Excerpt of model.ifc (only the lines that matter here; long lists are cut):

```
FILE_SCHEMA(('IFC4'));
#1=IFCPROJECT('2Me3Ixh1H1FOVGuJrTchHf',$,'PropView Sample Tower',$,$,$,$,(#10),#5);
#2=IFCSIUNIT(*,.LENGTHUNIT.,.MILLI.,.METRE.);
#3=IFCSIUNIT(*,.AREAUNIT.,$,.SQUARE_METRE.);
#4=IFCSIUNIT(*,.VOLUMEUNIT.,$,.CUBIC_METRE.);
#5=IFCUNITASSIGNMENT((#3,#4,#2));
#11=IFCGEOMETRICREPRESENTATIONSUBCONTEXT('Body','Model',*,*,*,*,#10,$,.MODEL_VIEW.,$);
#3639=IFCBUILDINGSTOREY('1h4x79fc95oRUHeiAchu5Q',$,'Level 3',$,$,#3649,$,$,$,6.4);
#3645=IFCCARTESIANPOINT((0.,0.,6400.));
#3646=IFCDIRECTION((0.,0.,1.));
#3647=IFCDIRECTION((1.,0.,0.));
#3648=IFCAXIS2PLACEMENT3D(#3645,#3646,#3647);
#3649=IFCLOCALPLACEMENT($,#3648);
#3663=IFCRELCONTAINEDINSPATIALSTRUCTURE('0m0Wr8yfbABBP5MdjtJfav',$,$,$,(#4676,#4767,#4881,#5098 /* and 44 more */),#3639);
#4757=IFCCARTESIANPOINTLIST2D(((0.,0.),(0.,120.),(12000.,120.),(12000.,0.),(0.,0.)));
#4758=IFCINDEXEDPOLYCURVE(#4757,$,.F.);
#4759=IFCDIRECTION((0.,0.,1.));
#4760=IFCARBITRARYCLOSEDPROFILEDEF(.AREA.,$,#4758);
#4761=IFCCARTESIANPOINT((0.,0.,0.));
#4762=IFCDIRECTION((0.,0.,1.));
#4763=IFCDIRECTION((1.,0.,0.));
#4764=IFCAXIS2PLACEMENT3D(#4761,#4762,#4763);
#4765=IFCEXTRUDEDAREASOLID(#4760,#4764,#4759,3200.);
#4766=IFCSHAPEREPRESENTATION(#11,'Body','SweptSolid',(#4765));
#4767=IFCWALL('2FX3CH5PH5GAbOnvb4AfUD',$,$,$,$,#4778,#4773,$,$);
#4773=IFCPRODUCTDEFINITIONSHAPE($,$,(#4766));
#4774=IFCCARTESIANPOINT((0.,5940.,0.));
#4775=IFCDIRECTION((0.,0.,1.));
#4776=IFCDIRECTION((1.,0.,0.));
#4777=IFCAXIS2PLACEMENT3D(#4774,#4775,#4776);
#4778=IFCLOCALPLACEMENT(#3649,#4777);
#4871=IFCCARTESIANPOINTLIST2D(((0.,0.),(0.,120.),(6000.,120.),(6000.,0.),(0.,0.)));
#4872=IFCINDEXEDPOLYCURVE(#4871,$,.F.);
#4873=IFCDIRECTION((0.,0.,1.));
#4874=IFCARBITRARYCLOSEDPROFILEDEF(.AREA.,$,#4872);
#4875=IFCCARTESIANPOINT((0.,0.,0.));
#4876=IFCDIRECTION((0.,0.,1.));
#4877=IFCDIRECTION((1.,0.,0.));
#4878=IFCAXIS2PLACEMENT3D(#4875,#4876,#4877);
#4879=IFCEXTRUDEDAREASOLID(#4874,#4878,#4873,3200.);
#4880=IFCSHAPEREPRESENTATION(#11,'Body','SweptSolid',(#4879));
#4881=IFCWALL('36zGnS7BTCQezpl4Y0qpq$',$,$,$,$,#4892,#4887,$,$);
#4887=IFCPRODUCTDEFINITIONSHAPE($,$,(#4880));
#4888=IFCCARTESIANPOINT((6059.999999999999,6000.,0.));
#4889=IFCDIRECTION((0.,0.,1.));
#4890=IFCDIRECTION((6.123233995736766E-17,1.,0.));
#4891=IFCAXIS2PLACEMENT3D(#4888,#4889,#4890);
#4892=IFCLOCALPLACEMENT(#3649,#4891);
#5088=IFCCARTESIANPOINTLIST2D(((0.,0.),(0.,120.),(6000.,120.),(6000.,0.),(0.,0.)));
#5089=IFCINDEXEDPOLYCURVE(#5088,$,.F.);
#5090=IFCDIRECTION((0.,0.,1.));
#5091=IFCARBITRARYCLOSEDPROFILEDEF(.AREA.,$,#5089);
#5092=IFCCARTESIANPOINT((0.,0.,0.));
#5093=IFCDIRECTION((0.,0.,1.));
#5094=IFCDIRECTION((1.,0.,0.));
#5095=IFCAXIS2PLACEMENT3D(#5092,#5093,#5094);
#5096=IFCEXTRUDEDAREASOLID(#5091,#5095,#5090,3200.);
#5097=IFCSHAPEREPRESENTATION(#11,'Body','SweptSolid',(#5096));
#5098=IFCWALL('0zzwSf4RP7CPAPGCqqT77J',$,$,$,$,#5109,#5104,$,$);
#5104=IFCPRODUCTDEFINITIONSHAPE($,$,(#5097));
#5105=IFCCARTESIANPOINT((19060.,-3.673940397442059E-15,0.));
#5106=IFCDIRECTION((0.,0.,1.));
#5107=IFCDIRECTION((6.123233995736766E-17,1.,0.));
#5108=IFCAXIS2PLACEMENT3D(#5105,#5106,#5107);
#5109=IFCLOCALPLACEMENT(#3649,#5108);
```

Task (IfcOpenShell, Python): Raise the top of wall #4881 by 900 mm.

```python
import ifcopenshell
import ifcopenshell.geom
import ifcopenshell.util.representation
import ifcopenshell.util.shape
import ifcopenshell.util.unit

model = ifcopenshell.open("model.ifc")
unit_scale = ifcopenshell.util.unit.calculate_unit_scale(model)
settings = ifcopenshell.geom.settings()


def volume(element):
    """Net volume in cubic metres, openings subtracted."""
    shape = ifcopenshell.geom.create_shape(settings, element)
    return ifcopenshell.util.shape.get_volume(shape.geometry)


wall = model.by_guid("36zGnS7BTCQezpl4Y0qpq$")
before = volume(wall)

body = ifcopenshell.util.representation.get_representation(wall, "Model", "Body")
solid = body.Items[0]
old_height = solid.Depth
solid.Depth += 0.9 / unit_scale
after = volume(wall)

print(f"height {old_height:g} -> {solid.Depth:g}, volume {before:.3f} -> {after:.3f} m3")

model.write("model_updated.ifc")
```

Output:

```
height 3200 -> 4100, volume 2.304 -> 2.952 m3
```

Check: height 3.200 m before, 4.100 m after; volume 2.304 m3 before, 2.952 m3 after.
